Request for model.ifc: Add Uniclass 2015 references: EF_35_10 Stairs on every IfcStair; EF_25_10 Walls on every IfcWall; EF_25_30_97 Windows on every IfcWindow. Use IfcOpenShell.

First a look at what the model holds.

```python
import ifcopenshell

model = ifcopenshell.open("model.ifc")
print(model.schema)
print("classifications:", [c.Name for c in model.by_type("IfcClassification")])
for ifc_class in ("IfcDoor", "IfcRoof", "IfcStair", "IfcWall", "IfcWindow"):
    print(ifc_class, len(model.by_type(ifc_class)))
```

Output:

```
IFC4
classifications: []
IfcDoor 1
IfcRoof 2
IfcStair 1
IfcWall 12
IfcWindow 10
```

```python
import ifcopenshell
import ifcopenshell.api.classification

model = ifcopenshell.open("model.ifc")

system = ifcopenshell.api.classification.add_classification(model, classification="Uniclass 2015")

codes = {
    "IfcStair": ("EF_35_10", "Stairs"),
    "IfcWall": ("EF_25_10", "Walls"),
    "IfcWindow": ("EF_25_30_97", "Windows"),
}
for ifc_class, (code, name) in codes.items():
    products = model.by_type(ifc_class)
    ifcopenshell.api.classification.add_reference(
        model, products=products, classification=system, identification=code, name=name
    )
    print(code, len(products))

model.write("model_edited.ifc")
```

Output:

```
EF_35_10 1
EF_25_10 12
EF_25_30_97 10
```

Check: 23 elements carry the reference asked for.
